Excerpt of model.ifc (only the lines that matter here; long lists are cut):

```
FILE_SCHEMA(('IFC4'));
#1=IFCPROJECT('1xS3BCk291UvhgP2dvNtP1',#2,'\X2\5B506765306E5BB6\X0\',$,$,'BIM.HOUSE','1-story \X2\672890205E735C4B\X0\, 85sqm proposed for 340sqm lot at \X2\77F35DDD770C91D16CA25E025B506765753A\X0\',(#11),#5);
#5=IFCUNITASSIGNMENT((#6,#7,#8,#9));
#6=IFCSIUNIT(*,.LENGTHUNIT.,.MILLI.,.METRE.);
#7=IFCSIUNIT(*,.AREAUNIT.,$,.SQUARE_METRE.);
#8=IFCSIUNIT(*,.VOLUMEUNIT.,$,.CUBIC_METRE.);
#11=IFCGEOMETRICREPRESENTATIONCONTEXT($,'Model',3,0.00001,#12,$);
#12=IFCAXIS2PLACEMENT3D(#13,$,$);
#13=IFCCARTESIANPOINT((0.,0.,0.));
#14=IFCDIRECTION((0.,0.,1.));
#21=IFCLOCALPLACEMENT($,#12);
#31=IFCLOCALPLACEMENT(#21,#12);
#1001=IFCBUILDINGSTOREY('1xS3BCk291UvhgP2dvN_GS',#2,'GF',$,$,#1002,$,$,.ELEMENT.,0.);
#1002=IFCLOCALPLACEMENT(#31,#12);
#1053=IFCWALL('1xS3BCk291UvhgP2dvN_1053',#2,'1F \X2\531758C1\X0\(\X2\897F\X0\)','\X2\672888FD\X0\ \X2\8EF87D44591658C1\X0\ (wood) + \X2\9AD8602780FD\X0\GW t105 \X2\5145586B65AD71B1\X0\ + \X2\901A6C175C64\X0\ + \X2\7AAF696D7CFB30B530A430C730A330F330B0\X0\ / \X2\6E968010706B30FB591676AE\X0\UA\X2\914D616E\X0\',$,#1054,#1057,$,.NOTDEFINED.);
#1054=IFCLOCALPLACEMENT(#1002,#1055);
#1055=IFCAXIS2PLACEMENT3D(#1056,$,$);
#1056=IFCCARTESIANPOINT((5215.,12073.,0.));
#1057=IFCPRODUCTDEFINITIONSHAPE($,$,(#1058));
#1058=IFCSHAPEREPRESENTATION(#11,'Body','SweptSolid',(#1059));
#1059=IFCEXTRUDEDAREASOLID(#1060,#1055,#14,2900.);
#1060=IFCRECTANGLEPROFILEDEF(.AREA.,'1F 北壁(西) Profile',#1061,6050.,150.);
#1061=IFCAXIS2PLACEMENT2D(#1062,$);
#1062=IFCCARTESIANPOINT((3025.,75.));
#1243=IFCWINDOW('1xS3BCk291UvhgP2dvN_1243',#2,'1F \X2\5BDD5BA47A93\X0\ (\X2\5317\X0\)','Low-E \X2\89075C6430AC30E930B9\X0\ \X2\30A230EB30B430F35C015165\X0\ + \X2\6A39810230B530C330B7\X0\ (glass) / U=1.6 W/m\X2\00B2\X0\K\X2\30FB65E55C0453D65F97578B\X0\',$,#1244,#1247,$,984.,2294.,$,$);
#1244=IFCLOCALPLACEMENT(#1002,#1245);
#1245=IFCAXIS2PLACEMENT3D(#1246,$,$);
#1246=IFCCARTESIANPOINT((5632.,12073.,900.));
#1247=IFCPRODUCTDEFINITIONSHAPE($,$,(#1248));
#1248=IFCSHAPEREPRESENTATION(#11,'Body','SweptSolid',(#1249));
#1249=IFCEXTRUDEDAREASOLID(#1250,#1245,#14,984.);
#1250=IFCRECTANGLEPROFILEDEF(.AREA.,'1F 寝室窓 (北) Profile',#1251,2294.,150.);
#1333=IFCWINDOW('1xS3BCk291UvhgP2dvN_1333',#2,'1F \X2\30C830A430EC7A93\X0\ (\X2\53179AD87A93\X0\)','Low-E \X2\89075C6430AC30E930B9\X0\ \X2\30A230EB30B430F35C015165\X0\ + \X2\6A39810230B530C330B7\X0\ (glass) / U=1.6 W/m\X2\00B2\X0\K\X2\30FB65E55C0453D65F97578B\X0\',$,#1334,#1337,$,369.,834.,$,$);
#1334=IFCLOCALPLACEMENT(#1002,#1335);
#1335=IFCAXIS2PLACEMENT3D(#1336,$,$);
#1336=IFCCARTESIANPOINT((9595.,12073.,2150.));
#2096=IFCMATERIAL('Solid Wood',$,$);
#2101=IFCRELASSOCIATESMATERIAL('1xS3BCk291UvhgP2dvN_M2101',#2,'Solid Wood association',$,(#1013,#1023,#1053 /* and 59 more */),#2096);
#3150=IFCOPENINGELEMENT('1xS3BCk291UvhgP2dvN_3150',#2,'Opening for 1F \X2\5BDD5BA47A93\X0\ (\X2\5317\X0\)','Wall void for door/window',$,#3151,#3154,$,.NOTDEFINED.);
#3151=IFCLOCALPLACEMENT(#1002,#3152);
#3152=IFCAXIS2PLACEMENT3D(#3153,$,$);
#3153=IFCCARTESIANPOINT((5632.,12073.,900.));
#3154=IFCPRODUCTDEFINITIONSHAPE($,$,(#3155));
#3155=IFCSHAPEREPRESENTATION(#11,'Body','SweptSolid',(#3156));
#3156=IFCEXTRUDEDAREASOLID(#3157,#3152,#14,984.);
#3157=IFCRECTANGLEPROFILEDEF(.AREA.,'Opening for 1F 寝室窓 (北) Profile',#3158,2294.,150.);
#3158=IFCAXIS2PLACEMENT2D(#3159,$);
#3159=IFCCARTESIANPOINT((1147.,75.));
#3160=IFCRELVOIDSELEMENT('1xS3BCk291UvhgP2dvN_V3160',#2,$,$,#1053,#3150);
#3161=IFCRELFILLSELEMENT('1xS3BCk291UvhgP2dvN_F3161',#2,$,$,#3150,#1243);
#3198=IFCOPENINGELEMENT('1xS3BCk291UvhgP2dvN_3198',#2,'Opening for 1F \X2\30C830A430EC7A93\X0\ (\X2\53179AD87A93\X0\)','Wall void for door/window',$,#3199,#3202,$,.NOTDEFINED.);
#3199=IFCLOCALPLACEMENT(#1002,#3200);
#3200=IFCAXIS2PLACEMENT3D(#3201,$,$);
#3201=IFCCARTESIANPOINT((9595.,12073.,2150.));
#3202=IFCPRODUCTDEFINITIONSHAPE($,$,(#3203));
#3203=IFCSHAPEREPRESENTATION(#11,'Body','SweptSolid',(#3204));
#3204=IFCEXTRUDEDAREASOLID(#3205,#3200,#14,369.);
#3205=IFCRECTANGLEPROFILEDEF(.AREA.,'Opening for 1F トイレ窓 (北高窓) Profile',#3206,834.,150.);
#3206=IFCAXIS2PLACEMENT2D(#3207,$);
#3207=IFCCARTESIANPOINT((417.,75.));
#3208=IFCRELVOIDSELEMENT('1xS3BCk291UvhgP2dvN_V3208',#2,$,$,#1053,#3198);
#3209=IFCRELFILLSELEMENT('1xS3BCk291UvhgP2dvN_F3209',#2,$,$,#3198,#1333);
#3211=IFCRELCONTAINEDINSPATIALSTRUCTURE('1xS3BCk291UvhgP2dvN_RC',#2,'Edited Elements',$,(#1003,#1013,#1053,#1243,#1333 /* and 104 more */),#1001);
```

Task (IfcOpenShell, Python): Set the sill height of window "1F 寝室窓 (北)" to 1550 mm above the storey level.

```python
import numpy as np
import ifcopenshell
import ifcopenshell.api.geometry
import ifcopenshell.geom
import ifcopenshell.util.element
import ifcopenshell.util.placement
import ifcopenshell.util.shape
import ifcopenshell.util.unit

model = ifcopenshell.open("model.ifc")
unit_scale = ifcopenshell.util.unit.calculate_unit_scale(model)

window = model.by_id(1243)
opening = window.FillsVoids[0].RelatingOpeningElement
storey = ifcopenshell.util.element.get_container(window, ifc_class="IfcBuildingStorey")
level = ifcopenshell.util.placement.get_local_placement(storey.ObjectPlacement)[2, 3]

# The opening's origin need not be at the sill, so measure its lowest point.
shape = ifcopenshell.geom.create_shape(ifcopenshell.geom.settings(), opening)
bottom = ifcopenshell.util.shape.get_shape_bottom_elevation(shape, shape.geometry) / unit_scale
dz = level + 1.55 / unit_scale - bottom

shift = np.array([0.0, 0.0, dz])
# The window is not placed relative to its opening, so move both.
for product in (opening, window):
    matrix = ifcopenshell.util.placement.get_local_placement(product.ObjectPlacement)
    matrix[:3, 3] += shift
    ifcopenshell.api.geometry.edit_object_placement(model, product=product, matrix=matrix, is_si=False)

print(f"moved by {dz * unit_scale:+.3f} m")

model.write("model_edited.ifc")
```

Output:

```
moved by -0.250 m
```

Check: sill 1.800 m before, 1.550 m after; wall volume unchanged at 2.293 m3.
